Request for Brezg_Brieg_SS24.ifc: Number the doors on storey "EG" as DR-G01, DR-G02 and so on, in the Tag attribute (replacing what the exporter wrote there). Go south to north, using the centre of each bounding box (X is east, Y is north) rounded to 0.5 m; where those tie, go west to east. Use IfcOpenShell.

First a look at what the model holds.

```python
import ifcopenshell
import ifcopenshell.util.element
import ifcopenshell.util.placement

model = ifcopenshell.open("Brezg_Brieg_SS24.ifc")
print(model.schema)
storey = next(s for s in model.by_type("IfcBuildingStorey") if s.Name == "EG")
doors = [e for e in ifcopenshell.util.element.get_decomposition(storey) if e.is_a("IfcDoor")]
for e in sorted(doors, key=lambda e: e.id()):
    origin = ifcopenshell.util.placement.get_local_placement(e.ObjectPlacement)[:3, 3]
    print(e.id(), e.Tag, e.Name, origin.round(2) + 0.0, sep=" | ")
```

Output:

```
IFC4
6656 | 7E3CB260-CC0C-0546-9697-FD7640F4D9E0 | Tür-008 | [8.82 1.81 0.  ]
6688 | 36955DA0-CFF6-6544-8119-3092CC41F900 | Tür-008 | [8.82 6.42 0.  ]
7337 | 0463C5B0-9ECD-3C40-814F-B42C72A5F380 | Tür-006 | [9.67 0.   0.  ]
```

```python
import ifcopenshell
import ifcopenshell.geom
import ifcopenshell.util.element
import ifcopenshell.util.shape

model = ifcopenshell.open("Brezg_Brieg_SS24.ifc")
settings = ifcopenshell.geom.settings()
settings.set("use-world-coords", True)


def centre(element):
    shape = ifcopenshell.geom.create_shape(settings, element)
    return ifcopenshell.util.shape.get_bbox_centroid(shape.geometry)


storey = next(s for s in model.by_type("IfcBuildingStorey") if s.Name == "EG")
doors = [e for e in ifcopenshell.util.element.get_decomposition(storey) if e.is_a("IfcDoor")]

# Insertion points can sit at a corner or the storey origin, so sort by the geometry (in metres).
centres = {e: centre(e) for e in doors}
doors.sort(key=lambda e: (round(centres[e][1] / 0.5), centres[e][0]))

for i, e in enumerate(doors, start=1):
    number = f"DR-G{i:02d}"
    e.Tag = number
    print(e.id(), number)

model.write("Brezg_Brieg_SS24_edited.ifc")
```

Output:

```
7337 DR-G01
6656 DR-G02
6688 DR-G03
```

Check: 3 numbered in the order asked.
